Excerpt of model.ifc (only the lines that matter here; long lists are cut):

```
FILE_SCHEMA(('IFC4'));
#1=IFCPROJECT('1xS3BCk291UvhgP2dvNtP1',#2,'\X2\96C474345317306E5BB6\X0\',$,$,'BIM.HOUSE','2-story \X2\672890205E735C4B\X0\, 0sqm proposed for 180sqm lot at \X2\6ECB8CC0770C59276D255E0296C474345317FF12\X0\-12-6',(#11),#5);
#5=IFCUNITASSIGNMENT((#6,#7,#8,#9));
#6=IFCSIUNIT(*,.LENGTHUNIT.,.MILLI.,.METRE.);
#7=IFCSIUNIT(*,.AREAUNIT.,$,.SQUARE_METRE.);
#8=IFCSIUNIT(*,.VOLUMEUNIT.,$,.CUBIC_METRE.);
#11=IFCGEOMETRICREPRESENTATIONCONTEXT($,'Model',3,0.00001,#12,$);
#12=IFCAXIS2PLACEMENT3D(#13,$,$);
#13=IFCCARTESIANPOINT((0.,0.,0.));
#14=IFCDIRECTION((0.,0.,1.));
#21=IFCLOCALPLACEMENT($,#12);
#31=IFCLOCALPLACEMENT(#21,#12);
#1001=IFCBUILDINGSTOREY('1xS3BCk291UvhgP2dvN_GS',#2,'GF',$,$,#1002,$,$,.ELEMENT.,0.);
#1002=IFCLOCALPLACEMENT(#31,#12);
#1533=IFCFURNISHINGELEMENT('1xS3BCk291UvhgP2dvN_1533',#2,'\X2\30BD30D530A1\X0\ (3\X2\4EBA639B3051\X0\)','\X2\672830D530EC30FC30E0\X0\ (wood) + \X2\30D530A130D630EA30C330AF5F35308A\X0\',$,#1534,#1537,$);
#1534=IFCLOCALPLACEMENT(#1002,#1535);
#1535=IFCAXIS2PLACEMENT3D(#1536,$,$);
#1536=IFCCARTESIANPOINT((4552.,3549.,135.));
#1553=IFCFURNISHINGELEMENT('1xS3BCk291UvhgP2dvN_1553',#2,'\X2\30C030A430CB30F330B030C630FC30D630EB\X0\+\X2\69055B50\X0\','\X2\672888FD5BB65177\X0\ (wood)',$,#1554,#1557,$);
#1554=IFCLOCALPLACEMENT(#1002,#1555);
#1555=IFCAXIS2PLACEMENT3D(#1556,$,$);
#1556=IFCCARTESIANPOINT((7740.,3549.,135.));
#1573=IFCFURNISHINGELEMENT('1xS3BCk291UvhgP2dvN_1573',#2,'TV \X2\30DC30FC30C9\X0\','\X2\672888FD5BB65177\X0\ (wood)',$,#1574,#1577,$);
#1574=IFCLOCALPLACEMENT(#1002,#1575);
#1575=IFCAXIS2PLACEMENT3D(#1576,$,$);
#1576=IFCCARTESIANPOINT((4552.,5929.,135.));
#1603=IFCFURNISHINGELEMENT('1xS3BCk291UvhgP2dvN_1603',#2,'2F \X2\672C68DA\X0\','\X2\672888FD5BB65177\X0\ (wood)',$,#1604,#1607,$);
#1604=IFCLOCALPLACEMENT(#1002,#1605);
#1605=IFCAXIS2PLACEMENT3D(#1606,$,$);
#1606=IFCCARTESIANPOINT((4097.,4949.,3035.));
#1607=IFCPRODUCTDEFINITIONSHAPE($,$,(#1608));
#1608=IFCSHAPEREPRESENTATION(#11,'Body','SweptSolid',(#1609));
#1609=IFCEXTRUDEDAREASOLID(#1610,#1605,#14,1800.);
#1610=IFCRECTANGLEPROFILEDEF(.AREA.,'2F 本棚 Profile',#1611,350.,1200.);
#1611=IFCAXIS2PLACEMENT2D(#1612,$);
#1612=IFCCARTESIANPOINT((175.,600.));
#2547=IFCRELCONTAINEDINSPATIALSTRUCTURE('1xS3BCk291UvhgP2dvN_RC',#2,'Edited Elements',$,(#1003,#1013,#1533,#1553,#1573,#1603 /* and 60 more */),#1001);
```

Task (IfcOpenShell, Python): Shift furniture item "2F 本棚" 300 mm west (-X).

```python
import ifcopenshell
import ifcopenshell.api.geometry
import ifcopenshell.util.placement

model = ifcopenshell.open("model.ifc")

item = model.by_guid("1xS3BCk291UvhgP2dvN_1603")
matrix = ifcopenshell.util.placement.get_local_placement(item.ObjectPlacement)
matrix[0, 3] -= 300.0
ifcopenshell.api.geometry.edit_object_placement(model, product=item, matrix=matrix, is_si=False)

print(ifcopenshell.util.placement.get_local_placement(item.ObjectPlacement).round(3) + 0.0)

model.write("model_v2.ifc")
```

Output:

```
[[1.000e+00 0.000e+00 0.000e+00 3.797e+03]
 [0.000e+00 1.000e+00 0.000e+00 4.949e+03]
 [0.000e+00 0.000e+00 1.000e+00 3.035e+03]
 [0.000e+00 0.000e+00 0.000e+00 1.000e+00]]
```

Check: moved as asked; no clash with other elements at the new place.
